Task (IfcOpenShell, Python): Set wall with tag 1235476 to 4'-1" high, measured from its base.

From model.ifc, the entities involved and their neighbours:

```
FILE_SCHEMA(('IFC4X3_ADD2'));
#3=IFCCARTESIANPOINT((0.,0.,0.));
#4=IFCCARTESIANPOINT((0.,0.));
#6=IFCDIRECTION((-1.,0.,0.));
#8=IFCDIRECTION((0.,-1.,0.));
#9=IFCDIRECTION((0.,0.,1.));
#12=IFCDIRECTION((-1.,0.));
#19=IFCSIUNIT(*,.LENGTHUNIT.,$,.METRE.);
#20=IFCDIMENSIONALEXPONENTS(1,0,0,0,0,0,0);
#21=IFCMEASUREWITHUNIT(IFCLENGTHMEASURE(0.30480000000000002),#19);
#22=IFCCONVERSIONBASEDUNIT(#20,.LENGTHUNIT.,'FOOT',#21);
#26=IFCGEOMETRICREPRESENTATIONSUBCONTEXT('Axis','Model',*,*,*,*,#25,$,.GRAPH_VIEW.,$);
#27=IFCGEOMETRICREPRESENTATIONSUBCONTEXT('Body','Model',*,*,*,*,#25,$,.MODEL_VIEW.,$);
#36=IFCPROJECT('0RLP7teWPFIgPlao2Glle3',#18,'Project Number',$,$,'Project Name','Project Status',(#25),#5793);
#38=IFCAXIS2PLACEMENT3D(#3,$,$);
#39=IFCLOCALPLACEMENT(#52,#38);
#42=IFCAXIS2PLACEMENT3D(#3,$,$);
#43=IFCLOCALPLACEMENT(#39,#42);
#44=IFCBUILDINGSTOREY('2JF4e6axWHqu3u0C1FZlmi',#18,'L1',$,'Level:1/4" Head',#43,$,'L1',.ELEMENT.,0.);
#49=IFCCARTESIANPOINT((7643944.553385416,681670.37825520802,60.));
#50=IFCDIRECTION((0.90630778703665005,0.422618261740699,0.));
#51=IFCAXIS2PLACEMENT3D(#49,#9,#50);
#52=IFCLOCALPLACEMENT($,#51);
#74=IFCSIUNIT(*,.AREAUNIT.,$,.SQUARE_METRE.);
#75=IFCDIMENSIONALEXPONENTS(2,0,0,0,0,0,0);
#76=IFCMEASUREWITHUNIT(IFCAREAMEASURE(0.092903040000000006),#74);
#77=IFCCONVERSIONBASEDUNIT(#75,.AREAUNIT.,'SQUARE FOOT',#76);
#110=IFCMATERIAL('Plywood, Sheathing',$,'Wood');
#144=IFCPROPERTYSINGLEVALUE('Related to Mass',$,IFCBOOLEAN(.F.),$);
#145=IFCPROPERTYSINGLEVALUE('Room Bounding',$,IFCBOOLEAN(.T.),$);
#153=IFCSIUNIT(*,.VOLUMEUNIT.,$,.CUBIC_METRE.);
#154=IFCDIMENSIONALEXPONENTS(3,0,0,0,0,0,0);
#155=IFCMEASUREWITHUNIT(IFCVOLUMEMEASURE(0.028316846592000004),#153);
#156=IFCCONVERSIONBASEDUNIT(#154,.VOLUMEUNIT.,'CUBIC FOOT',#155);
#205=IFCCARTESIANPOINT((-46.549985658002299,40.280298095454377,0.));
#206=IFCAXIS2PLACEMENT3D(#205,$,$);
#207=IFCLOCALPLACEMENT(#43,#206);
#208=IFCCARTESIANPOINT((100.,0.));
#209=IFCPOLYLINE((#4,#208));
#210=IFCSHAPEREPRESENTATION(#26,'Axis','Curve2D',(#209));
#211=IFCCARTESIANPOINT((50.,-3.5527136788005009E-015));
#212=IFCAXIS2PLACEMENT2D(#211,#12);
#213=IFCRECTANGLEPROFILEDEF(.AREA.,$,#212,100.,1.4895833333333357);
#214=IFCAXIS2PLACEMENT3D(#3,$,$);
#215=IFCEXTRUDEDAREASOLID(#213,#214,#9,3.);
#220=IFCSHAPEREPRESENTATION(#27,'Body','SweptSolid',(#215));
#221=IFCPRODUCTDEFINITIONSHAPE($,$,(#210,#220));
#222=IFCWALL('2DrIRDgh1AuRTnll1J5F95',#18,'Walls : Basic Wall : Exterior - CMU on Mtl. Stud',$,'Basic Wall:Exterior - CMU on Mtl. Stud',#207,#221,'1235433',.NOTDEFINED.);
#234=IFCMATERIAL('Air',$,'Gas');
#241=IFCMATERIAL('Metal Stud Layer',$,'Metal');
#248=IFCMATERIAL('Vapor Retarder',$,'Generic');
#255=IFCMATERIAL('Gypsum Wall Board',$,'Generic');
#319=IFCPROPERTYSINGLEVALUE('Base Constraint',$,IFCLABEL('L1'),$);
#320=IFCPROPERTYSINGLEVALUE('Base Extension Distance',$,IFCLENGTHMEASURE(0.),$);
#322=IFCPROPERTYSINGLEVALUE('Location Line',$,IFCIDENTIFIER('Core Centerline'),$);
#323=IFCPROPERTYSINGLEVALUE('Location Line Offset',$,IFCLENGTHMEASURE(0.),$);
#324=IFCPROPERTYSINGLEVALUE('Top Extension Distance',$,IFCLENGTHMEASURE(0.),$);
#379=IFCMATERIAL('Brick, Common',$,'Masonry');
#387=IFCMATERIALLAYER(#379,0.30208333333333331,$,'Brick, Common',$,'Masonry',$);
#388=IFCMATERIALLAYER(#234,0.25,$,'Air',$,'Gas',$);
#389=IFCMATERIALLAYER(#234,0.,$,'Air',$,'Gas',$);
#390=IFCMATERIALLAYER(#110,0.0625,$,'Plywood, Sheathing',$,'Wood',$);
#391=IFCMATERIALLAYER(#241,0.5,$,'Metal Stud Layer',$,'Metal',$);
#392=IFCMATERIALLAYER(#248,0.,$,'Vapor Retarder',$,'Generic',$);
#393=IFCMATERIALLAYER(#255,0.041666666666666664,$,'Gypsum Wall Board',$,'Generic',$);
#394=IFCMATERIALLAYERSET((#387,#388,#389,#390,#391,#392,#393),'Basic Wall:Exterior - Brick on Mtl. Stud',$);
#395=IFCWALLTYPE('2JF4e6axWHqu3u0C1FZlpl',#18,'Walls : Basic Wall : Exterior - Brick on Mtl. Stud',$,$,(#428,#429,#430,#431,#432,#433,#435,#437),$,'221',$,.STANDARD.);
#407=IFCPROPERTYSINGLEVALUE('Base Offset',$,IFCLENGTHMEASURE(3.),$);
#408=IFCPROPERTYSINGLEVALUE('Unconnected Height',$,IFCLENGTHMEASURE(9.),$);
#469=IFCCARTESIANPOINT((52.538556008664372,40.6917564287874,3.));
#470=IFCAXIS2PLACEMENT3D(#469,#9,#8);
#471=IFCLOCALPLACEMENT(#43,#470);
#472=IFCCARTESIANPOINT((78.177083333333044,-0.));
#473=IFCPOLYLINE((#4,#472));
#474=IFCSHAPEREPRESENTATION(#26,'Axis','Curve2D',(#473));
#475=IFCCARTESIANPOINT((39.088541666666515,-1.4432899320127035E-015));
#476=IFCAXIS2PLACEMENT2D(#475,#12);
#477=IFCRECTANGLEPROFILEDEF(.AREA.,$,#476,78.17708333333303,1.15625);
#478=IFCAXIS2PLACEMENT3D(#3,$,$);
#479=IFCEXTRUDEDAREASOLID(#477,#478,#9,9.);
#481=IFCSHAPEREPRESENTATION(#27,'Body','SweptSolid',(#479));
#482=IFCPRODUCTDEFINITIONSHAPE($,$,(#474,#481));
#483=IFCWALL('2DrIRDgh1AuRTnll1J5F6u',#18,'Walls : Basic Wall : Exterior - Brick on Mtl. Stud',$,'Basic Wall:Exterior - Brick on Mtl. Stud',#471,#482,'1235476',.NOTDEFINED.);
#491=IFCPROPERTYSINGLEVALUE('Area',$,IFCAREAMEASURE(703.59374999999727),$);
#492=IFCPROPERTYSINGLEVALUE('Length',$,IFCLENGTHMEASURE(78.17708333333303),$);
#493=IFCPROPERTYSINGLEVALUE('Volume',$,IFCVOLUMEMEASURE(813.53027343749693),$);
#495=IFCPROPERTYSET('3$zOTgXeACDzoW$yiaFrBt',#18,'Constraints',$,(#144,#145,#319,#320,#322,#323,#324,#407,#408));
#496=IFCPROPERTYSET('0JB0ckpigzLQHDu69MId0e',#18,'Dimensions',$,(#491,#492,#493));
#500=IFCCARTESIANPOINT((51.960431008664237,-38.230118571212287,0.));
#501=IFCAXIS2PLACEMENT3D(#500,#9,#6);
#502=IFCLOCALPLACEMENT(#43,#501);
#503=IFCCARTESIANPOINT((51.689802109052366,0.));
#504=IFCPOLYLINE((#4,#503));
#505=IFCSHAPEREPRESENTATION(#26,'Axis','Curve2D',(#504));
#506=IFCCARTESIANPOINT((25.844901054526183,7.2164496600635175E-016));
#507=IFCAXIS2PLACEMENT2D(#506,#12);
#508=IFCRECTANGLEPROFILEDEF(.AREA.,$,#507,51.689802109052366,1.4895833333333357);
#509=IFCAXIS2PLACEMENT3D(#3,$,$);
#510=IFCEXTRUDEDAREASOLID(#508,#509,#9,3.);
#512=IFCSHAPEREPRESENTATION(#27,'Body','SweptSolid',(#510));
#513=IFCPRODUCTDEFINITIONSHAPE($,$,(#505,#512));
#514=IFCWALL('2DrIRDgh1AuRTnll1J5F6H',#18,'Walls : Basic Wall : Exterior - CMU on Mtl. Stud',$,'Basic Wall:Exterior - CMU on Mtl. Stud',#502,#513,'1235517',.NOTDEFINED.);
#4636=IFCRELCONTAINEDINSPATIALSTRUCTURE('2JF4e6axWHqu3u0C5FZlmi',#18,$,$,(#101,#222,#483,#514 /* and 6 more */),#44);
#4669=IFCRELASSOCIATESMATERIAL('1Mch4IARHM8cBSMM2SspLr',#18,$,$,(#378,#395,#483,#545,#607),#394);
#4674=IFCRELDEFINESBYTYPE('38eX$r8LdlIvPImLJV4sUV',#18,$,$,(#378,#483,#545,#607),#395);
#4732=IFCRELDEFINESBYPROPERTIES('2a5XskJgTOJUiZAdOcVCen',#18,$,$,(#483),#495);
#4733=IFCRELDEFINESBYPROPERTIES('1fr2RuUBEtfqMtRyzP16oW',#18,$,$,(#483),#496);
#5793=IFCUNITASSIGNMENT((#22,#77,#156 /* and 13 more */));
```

```python
import ifcopenshell
import ifcopenshell.api.pset
import ifcopenshell.geom
import ifcopenshell.util.element
import ifcopenshell.util.representation
import ifcopenshell.util.shape
import ifcopenshell.util.unit

model = ifcopenshell.open("model.ifc")
unit_scale = ifcopenshell.util.unit.calculate_unit_scale(model)
area_scale = ifcopenshell.util.unit.calculate_unit_scale(model, "AREAUNIT")
volume_scale = ifcopenshell.util.unit.calculate_unit_scale(model, "VOLUMEUNIT")
settings = ifcopenshell.geom.settings()


def volume(element):
    """Net volume in cubic metres, openings subtracted."""
    shape = ifcopenshell.geom.create_shape(settings, element)
    return ifcopenshell.util.shape.get_volume(shape.geometry)


wall = model.by_guid("2DrIRDgh1AuRTnll1J5F6u")
before = volume(wall)

body = ifcopenshell.util.representation.get_representation(wall, "Model", "Body")
solid = body.Items[0]
old_height = solid.Depth
solid.Depth = 49 * 0.0254 / unit_scale
after = volume(wall)
thickness = 0.3524  # wall thickness in metres

# Update the stored height, areas and volumes.
pset = model.by_id(ifcopenshell.util.element.get_pset(wall, "Constraints", should_inherit=False)["id"])
ifcopenshell.api.pset.edit_pset(model, pset=pset, properties={
    "Unconnected Height": model.create_entity("IfcLengthMeasure", solid.Depth),
})
pset = model.by_id(ifcopenshell.util.element.get_pset(wall, "Dimensions", should_inherit=False)["id"])
ifcopenshell.api.pset.edit_pset(model, pset=pset, properties={
    "Area": model.create_entity("IfcAreaMeasure", after / thickness / area_scale),
    "Volume": model.create_entity("IfcVolumeMeasure", after / volume_scale),
})

print(f"height {old_height:g} -> {solid.Depth:g}, volume {before:.3f} -> {after:.3f} m3")

model.write("model-out.ifc")
```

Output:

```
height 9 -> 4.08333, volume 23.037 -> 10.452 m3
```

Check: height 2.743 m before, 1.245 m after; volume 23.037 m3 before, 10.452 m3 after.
